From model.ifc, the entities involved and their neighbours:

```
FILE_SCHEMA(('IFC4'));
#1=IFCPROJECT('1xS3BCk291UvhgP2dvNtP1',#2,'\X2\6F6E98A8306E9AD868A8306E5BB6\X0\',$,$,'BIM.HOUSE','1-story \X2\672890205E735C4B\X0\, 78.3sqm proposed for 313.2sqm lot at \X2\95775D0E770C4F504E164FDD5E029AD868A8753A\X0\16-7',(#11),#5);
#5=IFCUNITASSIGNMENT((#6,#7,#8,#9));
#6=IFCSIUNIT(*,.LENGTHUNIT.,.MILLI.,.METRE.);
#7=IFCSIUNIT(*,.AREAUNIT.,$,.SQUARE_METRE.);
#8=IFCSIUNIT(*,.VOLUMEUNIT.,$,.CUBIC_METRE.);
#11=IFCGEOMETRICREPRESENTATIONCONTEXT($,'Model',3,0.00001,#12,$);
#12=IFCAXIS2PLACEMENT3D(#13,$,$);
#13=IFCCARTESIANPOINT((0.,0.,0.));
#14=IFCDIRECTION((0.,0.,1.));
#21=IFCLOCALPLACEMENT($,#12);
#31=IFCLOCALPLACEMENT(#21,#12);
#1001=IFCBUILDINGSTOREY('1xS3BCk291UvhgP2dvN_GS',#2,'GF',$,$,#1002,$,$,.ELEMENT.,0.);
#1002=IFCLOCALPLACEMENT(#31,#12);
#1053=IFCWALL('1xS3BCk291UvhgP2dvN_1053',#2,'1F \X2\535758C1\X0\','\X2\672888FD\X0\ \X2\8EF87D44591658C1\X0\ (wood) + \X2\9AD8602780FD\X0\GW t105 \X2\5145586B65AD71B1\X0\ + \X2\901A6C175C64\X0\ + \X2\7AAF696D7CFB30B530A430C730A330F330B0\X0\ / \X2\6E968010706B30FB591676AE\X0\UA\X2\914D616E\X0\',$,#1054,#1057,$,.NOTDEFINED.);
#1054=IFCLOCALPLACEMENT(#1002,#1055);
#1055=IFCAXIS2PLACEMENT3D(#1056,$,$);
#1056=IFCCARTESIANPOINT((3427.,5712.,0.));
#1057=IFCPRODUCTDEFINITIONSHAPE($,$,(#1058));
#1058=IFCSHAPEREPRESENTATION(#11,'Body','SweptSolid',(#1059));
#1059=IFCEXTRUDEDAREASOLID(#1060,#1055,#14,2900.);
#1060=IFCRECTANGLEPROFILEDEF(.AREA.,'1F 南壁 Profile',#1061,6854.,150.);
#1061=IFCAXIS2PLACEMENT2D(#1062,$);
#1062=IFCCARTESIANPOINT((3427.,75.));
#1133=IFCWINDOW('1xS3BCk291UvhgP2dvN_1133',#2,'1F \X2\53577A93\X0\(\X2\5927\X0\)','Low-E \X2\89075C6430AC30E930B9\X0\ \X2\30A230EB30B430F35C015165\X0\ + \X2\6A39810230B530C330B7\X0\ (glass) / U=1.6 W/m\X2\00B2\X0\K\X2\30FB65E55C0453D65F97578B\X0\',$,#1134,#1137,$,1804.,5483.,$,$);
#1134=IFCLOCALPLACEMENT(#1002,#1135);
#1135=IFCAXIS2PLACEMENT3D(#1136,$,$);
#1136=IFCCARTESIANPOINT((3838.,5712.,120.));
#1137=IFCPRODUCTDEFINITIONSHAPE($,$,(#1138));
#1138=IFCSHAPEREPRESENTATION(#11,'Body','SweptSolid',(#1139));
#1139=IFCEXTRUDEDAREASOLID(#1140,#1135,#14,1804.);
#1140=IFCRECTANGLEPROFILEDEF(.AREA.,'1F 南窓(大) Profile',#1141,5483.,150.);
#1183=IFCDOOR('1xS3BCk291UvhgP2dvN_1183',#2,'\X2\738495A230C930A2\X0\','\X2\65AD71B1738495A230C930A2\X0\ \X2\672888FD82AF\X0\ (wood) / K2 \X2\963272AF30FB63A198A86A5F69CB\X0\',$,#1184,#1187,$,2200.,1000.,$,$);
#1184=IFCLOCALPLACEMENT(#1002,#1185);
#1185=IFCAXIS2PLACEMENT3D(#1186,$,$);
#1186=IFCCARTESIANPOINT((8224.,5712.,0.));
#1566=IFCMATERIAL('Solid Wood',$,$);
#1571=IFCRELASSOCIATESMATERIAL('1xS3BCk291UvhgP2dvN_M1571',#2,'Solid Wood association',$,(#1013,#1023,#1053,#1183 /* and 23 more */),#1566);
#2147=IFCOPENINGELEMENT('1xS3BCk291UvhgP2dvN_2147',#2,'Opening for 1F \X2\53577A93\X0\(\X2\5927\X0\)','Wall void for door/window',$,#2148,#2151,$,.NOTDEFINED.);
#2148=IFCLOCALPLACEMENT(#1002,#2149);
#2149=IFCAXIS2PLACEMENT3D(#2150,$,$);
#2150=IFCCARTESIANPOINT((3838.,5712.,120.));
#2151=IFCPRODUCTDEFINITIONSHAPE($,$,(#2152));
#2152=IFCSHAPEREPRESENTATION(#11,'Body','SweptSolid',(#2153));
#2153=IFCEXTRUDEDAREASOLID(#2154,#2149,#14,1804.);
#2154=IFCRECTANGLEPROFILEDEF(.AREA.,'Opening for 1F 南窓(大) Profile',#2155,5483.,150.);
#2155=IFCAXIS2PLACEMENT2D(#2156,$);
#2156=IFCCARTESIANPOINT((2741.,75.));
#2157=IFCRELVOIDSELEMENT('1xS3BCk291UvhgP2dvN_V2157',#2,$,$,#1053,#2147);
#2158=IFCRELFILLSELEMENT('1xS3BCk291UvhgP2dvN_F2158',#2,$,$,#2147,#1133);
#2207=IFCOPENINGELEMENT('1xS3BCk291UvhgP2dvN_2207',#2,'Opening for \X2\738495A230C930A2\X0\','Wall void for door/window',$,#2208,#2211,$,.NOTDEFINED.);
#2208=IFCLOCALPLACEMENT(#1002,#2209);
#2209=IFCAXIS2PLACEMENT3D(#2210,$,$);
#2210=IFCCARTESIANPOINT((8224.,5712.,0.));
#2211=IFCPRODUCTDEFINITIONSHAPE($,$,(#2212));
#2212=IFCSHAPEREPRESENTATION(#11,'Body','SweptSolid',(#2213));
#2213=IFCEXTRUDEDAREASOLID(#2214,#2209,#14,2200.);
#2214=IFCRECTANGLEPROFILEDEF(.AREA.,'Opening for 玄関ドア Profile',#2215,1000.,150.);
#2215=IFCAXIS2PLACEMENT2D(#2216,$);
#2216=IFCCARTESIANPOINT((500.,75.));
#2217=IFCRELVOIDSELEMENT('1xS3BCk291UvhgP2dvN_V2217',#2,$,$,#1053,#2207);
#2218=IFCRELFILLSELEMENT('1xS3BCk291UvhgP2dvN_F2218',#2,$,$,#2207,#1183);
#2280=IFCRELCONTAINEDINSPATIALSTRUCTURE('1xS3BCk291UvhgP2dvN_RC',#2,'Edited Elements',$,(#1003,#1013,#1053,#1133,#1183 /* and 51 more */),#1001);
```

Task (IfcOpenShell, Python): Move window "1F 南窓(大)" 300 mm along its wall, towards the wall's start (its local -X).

```python
import ifcopenshell
import ifcopenshell.api.geometry
import ifcopenshell.util.placement
import ifcopenshell.util.unit

model = ifcopenshell.open("model.ifc")
unit_scale = ifcopenshell.util.unit.calculate_unit_scale(model)

window = model.by_guid("1xS3BCk291UvhgP2dvN_1133")
opening = window.FillsVoids[0].RelatingOpeningElement
wall = opening.VoidsElements[0].RelatingBuildingElement

wall_matrix = ifcopenshell.util.placement.get_local_placement(wall.ObjectPlacement)
shift = wall_matrix[:3, 0] * -0.3 / unit_scale
before = ifcopenshell.util.placement.get_local_placement(window.ObjectPlacement)[:3, 3].copy()

# The window is not placed relative to its opening, so move both.
for product in (opening, window):
    matrix = ifcopenshell.util.placement.get_local_placement(product.ObjectPlacement)
    matrix[:3, 3] += shift
    ifcopenshell.api.geometry.edit_object_placement(model, product=product, matrix=matrix, is_si=False)

after = ifcopenshell.util.placement.get_local_placement(window.ObjectPlacement)[:3, 3]
print("window moved by", (after - before).round(3) + 0.0)

model.write("model_updated.ifc")
```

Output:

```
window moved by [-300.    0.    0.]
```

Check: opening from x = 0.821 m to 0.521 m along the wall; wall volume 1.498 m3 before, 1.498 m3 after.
